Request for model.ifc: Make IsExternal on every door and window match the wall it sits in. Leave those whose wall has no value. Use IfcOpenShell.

First a look at what the model holds.

```python
import ifcopenshell
import ifcopenshell.util.element

model = ifcopenshell.open("model.ifc")
print(model.schema)
seen = {}
for e in model.by_type("IfcDoor") + model.by_type("IfcWindow"):
    if not e.FillsVoids:
        continue
    host = e.FillsVoids[0].RelatingOpeningElement.VoidsElements[0].RelatingBuildingElement
    own = ifcopenshell.util.element.get_pset(e, f"Pset_{e.is_a()[3:].removesuffix('StandardCase')}Common", "IsExternal")
    wall = ifcopenshell.util.element.get_pset(host, "Pset_WallCommon", "IsExternal")
    seen[e.is_a(), own, wall] = seen.get((e.is_a(), own, wall), 0) + 1
for (cls, own, wall), count in sorted(seen.items(), key=str):
    print(count, cls, "IsExternal:", own, "| host wall:", wall)
```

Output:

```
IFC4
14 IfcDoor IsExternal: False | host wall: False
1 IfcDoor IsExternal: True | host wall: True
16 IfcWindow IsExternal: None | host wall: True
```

```python
import ifcopenshell
import ifcopenshell.api.pset
import ifcopenshell.util.element

model = ifcopenshell.open("model.ifc")

count = 0
for ifc_class, pset_name in (("IfcDoor", "Pset_DoorCommon"), ("IfcWindow", "Pset_WindowCommon")):
    for e in model.by_type(ifc_class):
        if not e.FillsVoids:
            continue
        host = e.FillsVoids[0].RelatingOpeningElement.VoidsElements[0].RelatingBuildingElement
        external = ifcopenshell.util.element.get_pset(host, "Pset_WallCommon", "IsExternal")
        if external is None or ifcopenshell.util.element.get_pset(e, pset_name, "IsExternal") == external:
            continue
        pset = ifcopenshell.api.pset.add_pset(model, product=e, name=pset_name)
        ifcopenshell.api.pset.edit_pset(model, pset=pset, properties={"IsExternal": external})
        count += 1

print(count, "updated")

model.write("model_updated.ifc")
```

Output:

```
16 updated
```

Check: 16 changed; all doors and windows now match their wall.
